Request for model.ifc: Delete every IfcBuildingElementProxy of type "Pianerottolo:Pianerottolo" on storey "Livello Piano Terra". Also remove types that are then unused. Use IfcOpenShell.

First a look at what the model holds.

```python
import ifcopenshell
import ifcopenshell.util.element

model = ifcopenshell.open("model.ifc")
print(model.schema)
storey = next(s for s in model.by_type("IfcBuildingStorey") if s.Name == "Livello Piano Terra")
proxies = [e for e in ifcopenshell.util.element.get_decomposition(storey) if e.is_a("IfcBuildingElementProxy")]
seen = {}
for e in proxies:
    element_type = ifcopenshell.util.element.get_type(e)
    name = element_type.Name if element_type not in (None, e) else None
    seen[name] = seen.get(name, 0) + 1
for name, count in sorted(seen.items(), key=str):
    print(count, "x", name)
```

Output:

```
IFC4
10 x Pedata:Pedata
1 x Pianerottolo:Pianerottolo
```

```python
import ifcopenshell
import ifcopenshell.api.root
import ifcopenshell.util.element

model = ifcopenshell.open("model.ifc")

storey = next(s for s in model.by_type("IfcBuildingStorey") if s.Name == "Livello Piano Terra")
proxies = [e for e in ifcopenshell.util.element.get_decomposition(storey) if e.is_a("IfcBuildingElementProxy")]
targets = [e for e in proxies if (t := ifcopenshell.util.element.get_type(e)) not in (None, e) and t.Name == "Pianerottolo:Pianerottolo"]
types = {ifcopenshell.util.element.get_type(e) for e in targets} - {None, *targets}

for e in targets:
    ifcopenshell.api.root.remove_product(model, product=e)
print(len(targets), "removed")

unused = [t for t in types if not ifcopenshell.util.element.get_types(t)]
for t in unused:
    ifcopenshell.api.root.remove_product(model, product=t)
print(len(unused), "unused types removed")

model.write("model-out.ifc")
```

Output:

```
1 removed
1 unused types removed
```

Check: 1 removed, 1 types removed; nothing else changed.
